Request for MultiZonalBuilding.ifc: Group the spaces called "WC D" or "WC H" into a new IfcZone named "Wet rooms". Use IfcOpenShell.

First a look at what the model holds.

```python
import ifcopenshell

model = ifcopenshell.open("MultiZonalBuilding.ifc")
print(model.schema)
seen = {}
for space in model.by_type("IfcSpace"):
    seen[space.LongName] = seen.get(space.LongName, 0) + 1
for name, count in sorted(seen.items(), key=str):
    print(count, "x", name)
print("zones:", [z.Name for z in model.by_type("IfcZone")][:20])
```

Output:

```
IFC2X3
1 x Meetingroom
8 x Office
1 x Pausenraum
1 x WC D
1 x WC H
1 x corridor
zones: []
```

```python
import ifcopenshell
import ifcopenshell.api.group
import ifcopenshell.api.root

model = ifcopenshell.open("MultiZonalBuilding.ifc")

names = {"WC D", "WC H"}
spaces = [s for s in model.by_type("IfcSpace") if s.LongName in names]

zone = ifcopenshell.api.root.create_entity(model, ifc_class="IfcZone", name="Wet rooms")
ifcopenshell.api.group.assign_group(model, products=spaces, group=zone)
print(len(spaces), "spaces in", zone.Name)

model.write("MultiZonalBuilding_edited.ifc")
```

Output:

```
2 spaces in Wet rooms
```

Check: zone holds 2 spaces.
